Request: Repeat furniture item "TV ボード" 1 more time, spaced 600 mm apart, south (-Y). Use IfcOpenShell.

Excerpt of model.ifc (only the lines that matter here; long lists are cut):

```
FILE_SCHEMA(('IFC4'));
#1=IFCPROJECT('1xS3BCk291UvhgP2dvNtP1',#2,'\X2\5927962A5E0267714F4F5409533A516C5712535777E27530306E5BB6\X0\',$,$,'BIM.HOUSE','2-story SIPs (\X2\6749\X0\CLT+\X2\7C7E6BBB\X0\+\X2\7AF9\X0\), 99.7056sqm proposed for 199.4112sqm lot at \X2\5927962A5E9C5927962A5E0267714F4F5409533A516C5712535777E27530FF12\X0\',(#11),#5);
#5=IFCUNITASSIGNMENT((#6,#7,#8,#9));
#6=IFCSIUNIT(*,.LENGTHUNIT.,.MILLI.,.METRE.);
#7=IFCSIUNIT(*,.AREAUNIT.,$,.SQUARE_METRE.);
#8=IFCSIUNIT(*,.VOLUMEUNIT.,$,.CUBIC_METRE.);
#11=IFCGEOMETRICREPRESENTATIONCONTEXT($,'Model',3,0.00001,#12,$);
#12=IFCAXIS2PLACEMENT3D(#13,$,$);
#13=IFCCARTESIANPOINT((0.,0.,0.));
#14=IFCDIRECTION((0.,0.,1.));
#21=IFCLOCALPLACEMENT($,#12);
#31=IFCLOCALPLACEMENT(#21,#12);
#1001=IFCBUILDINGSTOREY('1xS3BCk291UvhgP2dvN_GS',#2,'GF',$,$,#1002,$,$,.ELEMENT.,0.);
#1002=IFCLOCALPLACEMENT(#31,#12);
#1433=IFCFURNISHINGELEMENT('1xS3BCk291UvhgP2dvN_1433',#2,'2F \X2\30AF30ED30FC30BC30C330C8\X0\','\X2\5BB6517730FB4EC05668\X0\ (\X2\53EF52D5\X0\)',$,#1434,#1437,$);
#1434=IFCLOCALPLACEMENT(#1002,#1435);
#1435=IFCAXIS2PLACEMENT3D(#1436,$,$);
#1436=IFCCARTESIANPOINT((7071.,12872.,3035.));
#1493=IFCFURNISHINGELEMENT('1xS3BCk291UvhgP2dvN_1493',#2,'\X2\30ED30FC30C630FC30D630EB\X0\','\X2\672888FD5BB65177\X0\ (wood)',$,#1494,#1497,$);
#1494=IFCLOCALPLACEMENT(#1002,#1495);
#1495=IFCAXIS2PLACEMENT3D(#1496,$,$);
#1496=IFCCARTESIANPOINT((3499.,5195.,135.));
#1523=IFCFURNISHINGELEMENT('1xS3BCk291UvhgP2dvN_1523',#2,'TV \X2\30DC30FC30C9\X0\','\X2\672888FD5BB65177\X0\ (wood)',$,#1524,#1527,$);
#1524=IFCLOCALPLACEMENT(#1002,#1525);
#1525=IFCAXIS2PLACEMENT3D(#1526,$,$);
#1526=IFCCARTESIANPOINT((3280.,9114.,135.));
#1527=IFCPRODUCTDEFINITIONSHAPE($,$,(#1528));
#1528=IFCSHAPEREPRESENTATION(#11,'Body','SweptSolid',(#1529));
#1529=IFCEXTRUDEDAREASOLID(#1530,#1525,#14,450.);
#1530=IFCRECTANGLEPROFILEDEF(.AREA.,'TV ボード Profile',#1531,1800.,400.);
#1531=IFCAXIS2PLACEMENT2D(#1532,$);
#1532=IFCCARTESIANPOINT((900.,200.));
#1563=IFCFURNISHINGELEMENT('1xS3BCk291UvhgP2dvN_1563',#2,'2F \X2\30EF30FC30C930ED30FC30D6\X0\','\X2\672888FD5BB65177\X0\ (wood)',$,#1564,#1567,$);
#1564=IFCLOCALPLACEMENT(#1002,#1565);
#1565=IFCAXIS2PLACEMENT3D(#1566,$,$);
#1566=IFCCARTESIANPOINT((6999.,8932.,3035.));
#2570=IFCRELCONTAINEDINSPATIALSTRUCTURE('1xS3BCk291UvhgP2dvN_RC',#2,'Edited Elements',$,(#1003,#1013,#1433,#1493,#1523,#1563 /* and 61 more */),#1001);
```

```python
import numpy as np
import ifcopenshell
import ifcopenshell.api.geometry
import ifcopenshell.api.root
import ifcopenshell.util.element
import ifcopenshell.util.placement
import ifcopenshell.util.unit

model = ifcopenshell.open("model.ifc")
unit_scale = ifcopenshell.util.unit.calculate_unit_scale(model)


def reuse_history(source, copy):
    """copy_class also copies each property set's owner history, people and application; keep the originals."""
    for rel in copy.IsDefinedBy:
        if rel.is_a("IfcRelDefinesByProperties") and (history := rel.RelatingPropertyDefinition.OwnerHistory):
            rel.RelatingPropertyDefinition.OwnerHistory = source.OwnerHistory
            ifcopenshell.util.element.remove_deep2(model, history)


source = model.by_id(1523)
base = ifcopenshell.util.placement.get_local_placement(source.ObjectPlacement)
step = np.array([0.0, -1.0, 0.0]) * 0.6 / unit_scale

for i in range(1, 2):
    copy = ifcopenshell.api.root.copy_class(model, product=source)
    copy.Representation = ifcopenshell.util.element.copy_deep(
        model, source.Representation, exclude=["IfcGeometricRepresentationContext", "IfcRepresentationMap"]
    )
    reuse_history(source, copy)
    matrix = base.copy()
    matrix[:3, 3] += i * step
    print("added at", matrix[:3, 3].round(3) + 0.0)
    ifcopenshell.api.geometry.edit_object_placement(model, product=copy, matrix=matrix, is_si=False)

model.write("model_rev.ifc")
```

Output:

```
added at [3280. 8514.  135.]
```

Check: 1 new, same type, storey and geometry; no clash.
